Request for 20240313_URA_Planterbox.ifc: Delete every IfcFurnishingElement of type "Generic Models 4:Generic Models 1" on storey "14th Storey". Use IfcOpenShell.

First a look at what the model holds.

```python
import ifcopenshell
import ifcopenshell.util.element

model = ifcopenshell.open("20240313_URA_Planterbox.ifc")
print(model.schema)
storey = next(s for s in model.by_type("IfcBuildingStorey") if s.Name == "14th Storey")
furniture = [e for e in ifcopenshell.util.element.get_decomposition(storey) if e.is_a("IfcFurnishingElement")]
seen = {}
for e in furniture:
    element_type = ifcopenshell.util.element.get_type(e)
    name = element_type.Name if element_type not in (None, e) else None
    seen[name] = seen.get(name, 0) + 1
for name, count in sorted(seen.items(), key=str):
    print(count, "x", name)
```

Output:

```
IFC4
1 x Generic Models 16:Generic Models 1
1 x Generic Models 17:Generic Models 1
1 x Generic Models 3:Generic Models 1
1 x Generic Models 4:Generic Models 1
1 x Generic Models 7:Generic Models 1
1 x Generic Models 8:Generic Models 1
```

```python
import ifcopenshell
import ifcopenshell.api.root
import ifcopenshell.util.element

model = ifcopenshell.open("20240313_URA_Planterbox.ifc")

storey = next(s for s in model.by_type("IfcBuildingStorey") if s.Name == "14th Storey")
furniture = [e for e in ifcopenshell.util.element.get_decomposition(storey) if e.is_a("IfcFurnishingElement")]
targets = [e for e in furniture if (t := ifcopenshell.util.element.get_type(e)) not in (None, e) and t.Name == "Generic Models 4:Generic Models 1"]

for e in targets:
    ifcopenshell.api.root.remove_product(model, product=e)
print(len(targets), "removed")

model.write("20240313_URA_Planterbox_updated.ifc")
```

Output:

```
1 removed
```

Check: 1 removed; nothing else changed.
